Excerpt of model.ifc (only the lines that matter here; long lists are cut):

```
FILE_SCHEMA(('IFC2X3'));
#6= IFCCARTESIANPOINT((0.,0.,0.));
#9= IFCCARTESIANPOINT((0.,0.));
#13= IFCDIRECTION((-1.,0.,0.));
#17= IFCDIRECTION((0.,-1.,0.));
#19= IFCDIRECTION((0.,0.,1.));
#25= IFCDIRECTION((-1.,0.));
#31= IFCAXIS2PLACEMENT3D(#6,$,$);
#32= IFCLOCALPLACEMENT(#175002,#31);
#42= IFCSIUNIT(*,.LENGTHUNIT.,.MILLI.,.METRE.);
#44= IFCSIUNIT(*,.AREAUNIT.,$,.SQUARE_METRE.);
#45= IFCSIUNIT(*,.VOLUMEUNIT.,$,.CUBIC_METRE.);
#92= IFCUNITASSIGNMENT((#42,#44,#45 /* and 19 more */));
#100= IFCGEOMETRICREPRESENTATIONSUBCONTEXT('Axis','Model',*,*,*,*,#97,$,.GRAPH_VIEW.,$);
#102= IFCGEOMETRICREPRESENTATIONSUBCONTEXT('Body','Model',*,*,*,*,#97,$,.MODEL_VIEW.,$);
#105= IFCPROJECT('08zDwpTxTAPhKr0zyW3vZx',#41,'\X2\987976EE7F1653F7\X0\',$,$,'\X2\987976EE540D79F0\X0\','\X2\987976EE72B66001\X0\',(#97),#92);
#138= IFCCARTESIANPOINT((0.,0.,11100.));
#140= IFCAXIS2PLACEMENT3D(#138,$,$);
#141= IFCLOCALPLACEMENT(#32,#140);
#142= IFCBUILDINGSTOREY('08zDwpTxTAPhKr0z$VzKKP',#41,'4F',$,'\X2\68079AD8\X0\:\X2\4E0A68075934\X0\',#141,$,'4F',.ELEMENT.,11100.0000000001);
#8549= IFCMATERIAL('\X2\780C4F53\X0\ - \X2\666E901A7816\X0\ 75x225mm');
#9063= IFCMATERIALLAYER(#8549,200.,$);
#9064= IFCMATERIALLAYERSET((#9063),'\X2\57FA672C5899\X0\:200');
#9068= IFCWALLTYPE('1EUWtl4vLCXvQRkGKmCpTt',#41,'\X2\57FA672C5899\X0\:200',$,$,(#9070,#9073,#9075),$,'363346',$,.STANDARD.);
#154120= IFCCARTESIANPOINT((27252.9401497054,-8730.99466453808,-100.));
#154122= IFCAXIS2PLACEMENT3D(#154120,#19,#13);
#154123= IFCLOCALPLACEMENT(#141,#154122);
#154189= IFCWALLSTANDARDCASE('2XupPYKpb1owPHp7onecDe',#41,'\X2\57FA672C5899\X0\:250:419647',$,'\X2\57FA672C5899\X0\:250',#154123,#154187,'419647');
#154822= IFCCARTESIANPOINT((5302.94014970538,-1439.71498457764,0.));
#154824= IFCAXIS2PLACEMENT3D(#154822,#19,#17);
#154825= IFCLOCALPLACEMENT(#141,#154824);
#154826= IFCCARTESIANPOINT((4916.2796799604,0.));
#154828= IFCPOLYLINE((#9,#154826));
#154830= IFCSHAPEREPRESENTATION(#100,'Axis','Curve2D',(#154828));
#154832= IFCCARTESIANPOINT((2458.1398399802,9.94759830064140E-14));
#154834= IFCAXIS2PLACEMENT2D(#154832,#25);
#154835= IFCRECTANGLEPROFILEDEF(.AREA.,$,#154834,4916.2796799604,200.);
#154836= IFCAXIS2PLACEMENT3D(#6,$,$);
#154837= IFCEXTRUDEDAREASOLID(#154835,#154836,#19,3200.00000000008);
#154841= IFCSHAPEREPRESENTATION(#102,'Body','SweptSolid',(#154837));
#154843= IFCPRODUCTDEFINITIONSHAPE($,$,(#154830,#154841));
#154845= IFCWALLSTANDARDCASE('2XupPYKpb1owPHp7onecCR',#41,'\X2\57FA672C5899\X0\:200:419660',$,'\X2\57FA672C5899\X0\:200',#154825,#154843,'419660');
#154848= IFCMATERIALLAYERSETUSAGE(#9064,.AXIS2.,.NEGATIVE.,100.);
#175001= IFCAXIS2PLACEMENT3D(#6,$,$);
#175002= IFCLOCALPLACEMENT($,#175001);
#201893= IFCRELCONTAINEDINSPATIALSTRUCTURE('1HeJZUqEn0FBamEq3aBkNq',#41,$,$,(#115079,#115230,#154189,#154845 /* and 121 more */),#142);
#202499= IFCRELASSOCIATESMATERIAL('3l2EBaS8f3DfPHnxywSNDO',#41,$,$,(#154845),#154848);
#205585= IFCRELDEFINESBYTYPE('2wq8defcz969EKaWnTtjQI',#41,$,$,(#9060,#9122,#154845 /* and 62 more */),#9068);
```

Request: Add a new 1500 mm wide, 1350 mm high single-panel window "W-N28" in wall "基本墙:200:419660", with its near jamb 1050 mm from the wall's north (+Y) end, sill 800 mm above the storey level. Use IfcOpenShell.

```python
import numpy as np
import ifcopenshell
import ifcopenshell.api.feature
import ifcopenshell.api.geometry
import ifcopenshell.api.root
import ifcopenshell.api.spatial
import ifcopenshell.api.type
import ifcopenshell.geom
import ifcopenshell.util.element
import ifcopenshell.util.placement
import ifcopenshell.util.representation
import ifcopenshell.util.shape
import ifcopenshell.util.unit

model = ifcopenshell.open("model.ifc")
unit_scale = ifcopenshell.util.unit.calculate_unit_scale(model)
settings = ifcopenshell.geom.settings()


def volume(element):
    """Net volume in cubic metres, openings subtracted."""
    shape = ifcopenshell.geom.create_shape(settings, element)
    return ifcopenshell.util.shape.get_volume(shape.geometry)


wall = model.by_guid("2XupPYKpb1owPHp7onecCR")
storey = ifcopenshell.util.element.get_container(wall, ifc_class="IfcBuildingStorey")
context = ifcopenshell.util.representation.get_context(model, "Model", "Body", "MODEL_VIEW")
before = volume(wall)

width, height, from_end, sill = 1.5, 1.35, 1.05, 0.8  # metres

# The wall runs along its own X axis, and the end named is its -X end.
wall_shape = ifcopenshell.geom.create_shape(settings, wall)
x, y, z = ifcopenshell.util.shape.get_vertices(wall_shape.geometry).T
start = x.min() + from_end
face, thickness = float(y.min()), float(y.max() - y.min())
wall_matrix = ifcopenshell.util.placement.get_local_placement(wall.ObjectPlacement)
level = ifcopenshell.util.placement.get_local_placement(storey.ObjectPlacement)[2, 3]


def in_wall(x, y):
    """Placement at x, y metres in the wall's axes, at sill height."""
    matrix = wall_matrix.copy()
    matrix[:, 3] = wall_matrix @ np.array([x / unit_scale, y / unit_scale, 0.0, 1.0])
    matrix[2, 3] = level + sill / unit_scale
    return matrix


# Opening: a box that overshoots both wall faces by 50 mm.
opening = ifcopenshell.api.root.create_entity(model, ifc_class="IfcOpeningElement")
box = ifcopenshell.api.geometry.add_wall_representation(
    model, context=context, length=width, height=height, thickness=thickness + 0.1
)
ifcopenshell.api.geometry.assign_representation(model, product=opening, representation=box)
ifcopenshell.api.geometry.edit_object_placement(model, product=opening, matrix=in_wall(start, face - 0.05), is_si=False)
ifcopenshell.api.feature.add_feature(model, feature=opening, element=wall)

window = ifcopenshell.api.root.create_entity(model, ifc_class="IfcWindow", name="W-N28")
window.OverallWidth, window.OverallHeight = width / unit_scale, height / unit_scale
body = ifcopenshell.api.geometry.add_window_representation(
    model,
    context=context,
    overall_width=window.OverallWidth,
    overall_height=window.OverallHeight,
    partition_type="SINGLE_PANEL",
)
ifcopenshell.api.geometry.assign_representation(model, product=window, representation=body)
ifcopenshell.api.spatial.assign_container(model, products=[window], relating_structure=storey)
fills = ifcopenshell.api.feature.add_filling(model, opening=opening, element=window)
fills.OwnerHistory = window.OwnerHistory  # required in IFC2X3

# IFC2X3 keeps the operation on the window style.
style = ifcopenshell.api.root.create_entity(model, ifc_class="IfcWindowStyle", name="W-N28")
style.OperationType, style.ConstructionType = "SINGLE_PANEL", "NOTDEFINED"
style.ParameterTakesPrecedence = style.Sizeable = False
ifcopenshell.api.type.assign_type(model, related_objects=[window], relating_type=style)

# Centre the window in the wall's thickness.
ifcopenshell.api.geometry.edit_object_placement(model, product=window, matrix=in_wall(start, face), is_si=False)
window_shape = ifcopenshell.geom.create_shape(settings, window)
depth = ifcopenshell.util.shape.get_vertices(window_shape.geometry)[:, 1]
offset = face + thickness / 2 - (depth.min() + depth.max()) / 2
ifcopenshell.api.geometry.edit_object_placement(model, product=window, matrix=in_wall(start, offset), is_si=False)

after = volume(wall)

print(f"wall volume {before:.3f} -> {after:.3f} m3")

model.write("model_edited.ifc")
```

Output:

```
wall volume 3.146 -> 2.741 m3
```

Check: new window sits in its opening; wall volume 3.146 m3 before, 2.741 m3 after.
